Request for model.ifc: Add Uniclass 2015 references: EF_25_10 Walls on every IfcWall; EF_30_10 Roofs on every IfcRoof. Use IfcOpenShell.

First a look at what the model holds.

```python
import ifcopenshell

model = ifcopenshell.open("model.ifc")
print(model.schema)
print("classifications:", [c.Name for c in model.by_type("IfcClassification")])
for ifc_class in ("IfcDoor", "IfcRoof", "IfcStair", "IfcWall", "IfcWindow"):
    print(ifc_class, len(model.by_type(ifc_class)))
```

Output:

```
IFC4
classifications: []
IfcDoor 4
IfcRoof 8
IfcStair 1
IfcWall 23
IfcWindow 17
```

```python
import ifcopenshell
import ifcopenshell.api.classification

model = ifcopenshell.open("model.ifc")

system = ifcopenshell.api.classification.add_classification(model, classification="Uniclass 2015")

codes = {
    "IfcWall": ("EF_25_10", "Walls"),
    "IfcRoof": ("EF_30_10", "Roofs"),
}
for ifc_class, (code, name) in codes.items():
    products = model.by_type(ifc_class)
    ifcopenshell.api.classification.add_reference(
        model, products=products, classification=system, identification=code, name=name
    )
    print(code, len(products))

model.write("model-out.ifc")
```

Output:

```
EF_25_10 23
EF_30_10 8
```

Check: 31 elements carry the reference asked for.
